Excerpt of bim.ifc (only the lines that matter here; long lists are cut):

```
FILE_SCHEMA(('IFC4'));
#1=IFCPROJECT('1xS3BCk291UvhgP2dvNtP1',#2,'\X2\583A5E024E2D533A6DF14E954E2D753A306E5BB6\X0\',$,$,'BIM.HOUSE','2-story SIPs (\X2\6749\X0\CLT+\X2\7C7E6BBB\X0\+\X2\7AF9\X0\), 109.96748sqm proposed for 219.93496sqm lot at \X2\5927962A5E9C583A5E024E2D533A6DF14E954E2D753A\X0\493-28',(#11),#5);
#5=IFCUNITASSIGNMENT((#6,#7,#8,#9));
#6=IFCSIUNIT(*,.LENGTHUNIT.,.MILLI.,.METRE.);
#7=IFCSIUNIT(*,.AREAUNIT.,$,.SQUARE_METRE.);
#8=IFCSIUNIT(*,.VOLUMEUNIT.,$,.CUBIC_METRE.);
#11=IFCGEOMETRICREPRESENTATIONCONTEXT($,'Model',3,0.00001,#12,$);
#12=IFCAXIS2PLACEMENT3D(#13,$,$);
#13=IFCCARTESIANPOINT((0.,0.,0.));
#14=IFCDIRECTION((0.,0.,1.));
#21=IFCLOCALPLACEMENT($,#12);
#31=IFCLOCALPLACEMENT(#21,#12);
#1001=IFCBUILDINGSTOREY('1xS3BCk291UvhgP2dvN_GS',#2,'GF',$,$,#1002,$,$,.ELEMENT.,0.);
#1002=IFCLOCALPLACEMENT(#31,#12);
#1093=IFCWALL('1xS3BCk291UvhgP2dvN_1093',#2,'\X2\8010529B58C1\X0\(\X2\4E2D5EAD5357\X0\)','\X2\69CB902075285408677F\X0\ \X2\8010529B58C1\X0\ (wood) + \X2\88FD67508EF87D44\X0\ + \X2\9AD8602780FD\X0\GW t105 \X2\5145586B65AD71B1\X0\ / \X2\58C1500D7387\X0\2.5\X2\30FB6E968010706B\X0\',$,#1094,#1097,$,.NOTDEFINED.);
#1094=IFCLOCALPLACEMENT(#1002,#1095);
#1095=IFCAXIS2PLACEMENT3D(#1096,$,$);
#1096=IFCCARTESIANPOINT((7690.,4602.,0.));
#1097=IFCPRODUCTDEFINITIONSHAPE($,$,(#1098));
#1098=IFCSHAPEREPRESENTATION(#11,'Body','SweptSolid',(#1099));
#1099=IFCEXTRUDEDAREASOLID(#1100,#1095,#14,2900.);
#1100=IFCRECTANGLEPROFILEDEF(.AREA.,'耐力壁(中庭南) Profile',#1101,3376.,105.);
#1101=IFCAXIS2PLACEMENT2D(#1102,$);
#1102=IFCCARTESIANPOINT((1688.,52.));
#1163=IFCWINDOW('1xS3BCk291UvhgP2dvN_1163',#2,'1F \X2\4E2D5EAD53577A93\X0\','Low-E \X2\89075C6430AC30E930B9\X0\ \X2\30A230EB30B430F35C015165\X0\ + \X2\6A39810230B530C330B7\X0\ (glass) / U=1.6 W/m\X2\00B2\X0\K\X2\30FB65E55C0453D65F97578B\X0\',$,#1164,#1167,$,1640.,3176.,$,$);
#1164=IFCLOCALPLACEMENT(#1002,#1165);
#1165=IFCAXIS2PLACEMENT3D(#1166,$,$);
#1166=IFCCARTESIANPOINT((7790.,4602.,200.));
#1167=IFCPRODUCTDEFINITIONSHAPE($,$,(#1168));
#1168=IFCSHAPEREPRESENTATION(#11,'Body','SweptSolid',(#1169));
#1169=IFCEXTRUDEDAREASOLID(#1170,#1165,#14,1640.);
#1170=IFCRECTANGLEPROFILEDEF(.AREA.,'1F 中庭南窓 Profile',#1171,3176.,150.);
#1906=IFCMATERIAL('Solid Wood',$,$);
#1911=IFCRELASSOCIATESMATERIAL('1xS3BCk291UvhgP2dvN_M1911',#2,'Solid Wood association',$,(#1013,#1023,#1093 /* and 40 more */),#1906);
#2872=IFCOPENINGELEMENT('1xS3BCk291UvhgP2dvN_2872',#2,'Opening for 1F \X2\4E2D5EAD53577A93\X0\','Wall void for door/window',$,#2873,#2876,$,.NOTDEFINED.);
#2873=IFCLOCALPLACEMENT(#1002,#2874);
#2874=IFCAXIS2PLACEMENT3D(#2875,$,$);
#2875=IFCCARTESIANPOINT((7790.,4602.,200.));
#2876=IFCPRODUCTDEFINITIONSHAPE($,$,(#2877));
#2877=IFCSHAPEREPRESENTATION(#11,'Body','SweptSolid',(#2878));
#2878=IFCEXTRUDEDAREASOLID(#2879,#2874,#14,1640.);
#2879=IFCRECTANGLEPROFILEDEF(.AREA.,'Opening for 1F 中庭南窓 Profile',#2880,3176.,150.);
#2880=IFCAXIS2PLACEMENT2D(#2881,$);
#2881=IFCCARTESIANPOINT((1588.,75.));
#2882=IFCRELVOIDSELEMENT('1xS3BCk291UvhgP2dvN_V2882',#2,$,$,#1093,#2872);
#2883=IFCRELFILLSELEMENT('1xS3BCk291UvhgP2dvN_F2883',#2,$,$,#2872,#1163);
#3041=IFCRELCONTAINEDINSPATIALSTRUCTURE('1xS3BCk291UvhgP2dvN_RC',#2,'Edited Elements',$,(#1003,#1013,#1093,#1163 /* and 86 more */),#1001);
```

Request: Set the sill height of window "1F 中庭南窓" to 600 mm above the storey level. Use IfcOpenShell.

```python
import numpy as np
import ifcopenshell
import ifcopenshell.api.geometry
import ifcopenshell.geom
import ifcopenshell.util.element
import ifcopenshell.util.placement
import ifcopenshell.util.shape
import ifcopenshell.util.unit

model = ifcopenshell.open("bim.ifc")
unit_scale = ifcopenshell.util.unit.calculate_unit_scale(model)

window = model.by_guid("1xS3BCk291UvhgP2dvN_1163")
opening = window.FillsVoids[0].RelatingOpeningElement
storey = ifcopenshell.util.element.get_container(window, ifc_class="IfcBuildingStorey")
level = ifcopenshell.util.placement.get_local_placement(storey.ObjectPlacement)[2, 3]

# The opening's origin need not be at the sill, so measure its lowest point.
shape = ifcopenshell.geom.create_shape(ifcopenshell.geom.settings(), opening)
bottom = ifcopenshell.util.shape.get_shape_bottom_elevation(shape, shape.geometry) / unit_scale
dz = level + 0.6 / unit_scale - bottom

shift = np.array([0.0, 0.0, dz])
# The window is not placed relative to its opening, so move both.
for product in (opening, window):
    matrix = ifcopenshell.util.placement.get_local_placement(product.ObjectPlacement)
    matrix[:3, 3] += shift
    ifcopenshell.api.geometry.edit_object_placement(model, product=product, matrix=matrix, is_si=False)

print(f"moved by {dz * unit_scale:+.3f} m")

model.write("bim_edited.ifc")
```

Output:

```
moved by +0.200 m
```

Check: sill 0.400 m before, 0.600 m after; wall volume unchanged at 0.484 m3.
